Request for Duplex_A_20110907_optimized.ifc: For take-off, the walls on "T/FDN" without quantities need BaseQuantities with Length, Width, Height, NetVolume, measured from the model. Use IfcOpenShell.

First a look at what the model holds.

```python
import ifcopenshell
import ifcopenshell.util.element
import ifcopenshell.util.unit

model = ifcopenshell.open("Duplex_A_20110907_optimized.ifc")
print(model.schema)
for unit_type in ("LENGTHUNIT", "AREAUNIT", "VOLUMEUNIT"):
    print(unit_type, ifcopenshell.util.unit.calculate_unit_scale(model, unit_type))
storey = next(s for s in model.by_type("IfcBuildingStorey") if s.Name == "T/FDN")
walls = [e for e in ifcopenshell.util.element.get_decomposition(storey) if e.is_a("IfcWall")]
for e in sorted(walls, key=lambda e: e.id()):
    print(e.id(), e.is_a(), e.Name, list(ifcopenshell.util.element.get_psets(e, qtos_only=True)), sep=" | ")
```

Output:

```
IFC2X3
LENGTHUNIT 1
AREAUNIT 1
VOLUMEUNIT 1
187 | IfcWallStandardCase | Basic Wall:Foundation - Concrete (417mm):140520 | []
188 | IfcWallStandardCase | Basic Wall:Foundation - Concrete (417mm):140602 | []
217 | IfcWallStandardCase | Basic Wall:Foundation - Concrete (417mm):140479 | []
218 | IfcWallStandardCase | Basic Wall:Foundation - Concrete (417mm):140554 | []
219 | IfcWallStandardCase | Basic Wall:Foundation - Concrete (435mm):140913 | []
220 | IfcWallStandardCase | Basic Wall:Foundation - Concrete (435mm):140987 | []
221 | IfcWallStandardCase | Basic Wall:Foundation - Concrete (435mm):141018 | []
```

```python
import ifcopenshell
import ifcopenshell.api.pset
import ifcopenshell.geom
import ifcopenshell.util.element
import ifcopenshell.util.shape
import ifcopenshell.util.unit

model = ifcopenshell.open("Duplex_A_20110907_optimized.ifc")
unit_scale = ifcopenshell.util.unit.calculate_unit_scale(model)
volume_scale = ifcopenshell.util.unit.calculate_unit_scale(model, "VOLUMEUNIT")
settings = ifcopenshell.geom.settings()

storey = next(s for s in model.by_type("IfcBuildingStorey") if s.Name == "T/FDN")
walls = [e for e in ifcopenshell.util.element.get_decomposition(storey) if e.is_a("IfcWall")]

for e in sorted(walls, key=lambda e: e.id()):
    if ifcopenshell.util.element.get_psets(e, qtos_only=True, should_inherit=False):
        continue
    # Geometry comes back in metres, in the element's own axes.
    shape = ifcopenshell.geom.create_shape(settings, e)
    values = {
        "Length": ifcopenshell.util.shape.get_x(shape.geometry) / unit_scale,
        "Width": ifcopenshell.util.shape.get_y(shape.geometry) / unit_scale,
        "Height": ifcopenshell.util.shape.get_z(shape.geometry) / unit_scale,
        "NetVolume": ifcopenshell.util.shape.get_volume(shape.geometry) / volume_scale,
    }
    qto = ifcopenshell.api.pset.add_qto(model, product=e, name="BaseQuantities")
    ifcopenshell.api.pset.edit_qto(model, qto=qto, properties=values)
    print(e.id(), {k: round(v, 3) for k, v in values.items()})

model.write("Duplex_A_20110907_optimized_updated.ifc")
```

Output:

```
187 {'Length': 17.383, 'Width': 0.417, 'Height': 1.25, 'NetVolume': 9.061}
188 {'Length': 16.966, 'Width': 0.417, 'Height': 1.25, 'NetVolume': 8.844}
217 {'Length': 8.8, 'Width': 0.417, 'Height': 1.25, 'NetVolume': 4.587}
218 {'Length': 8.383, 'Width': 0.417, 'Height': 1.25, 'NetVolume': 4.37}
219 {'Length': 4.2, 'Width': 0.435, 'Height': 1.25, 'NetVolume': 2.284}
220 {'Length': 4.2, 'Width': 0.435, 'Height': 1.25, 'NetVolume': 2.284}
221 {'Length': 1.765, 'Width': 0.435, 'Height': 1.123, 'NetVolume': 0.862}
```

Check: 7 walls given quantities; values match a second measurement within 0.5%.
